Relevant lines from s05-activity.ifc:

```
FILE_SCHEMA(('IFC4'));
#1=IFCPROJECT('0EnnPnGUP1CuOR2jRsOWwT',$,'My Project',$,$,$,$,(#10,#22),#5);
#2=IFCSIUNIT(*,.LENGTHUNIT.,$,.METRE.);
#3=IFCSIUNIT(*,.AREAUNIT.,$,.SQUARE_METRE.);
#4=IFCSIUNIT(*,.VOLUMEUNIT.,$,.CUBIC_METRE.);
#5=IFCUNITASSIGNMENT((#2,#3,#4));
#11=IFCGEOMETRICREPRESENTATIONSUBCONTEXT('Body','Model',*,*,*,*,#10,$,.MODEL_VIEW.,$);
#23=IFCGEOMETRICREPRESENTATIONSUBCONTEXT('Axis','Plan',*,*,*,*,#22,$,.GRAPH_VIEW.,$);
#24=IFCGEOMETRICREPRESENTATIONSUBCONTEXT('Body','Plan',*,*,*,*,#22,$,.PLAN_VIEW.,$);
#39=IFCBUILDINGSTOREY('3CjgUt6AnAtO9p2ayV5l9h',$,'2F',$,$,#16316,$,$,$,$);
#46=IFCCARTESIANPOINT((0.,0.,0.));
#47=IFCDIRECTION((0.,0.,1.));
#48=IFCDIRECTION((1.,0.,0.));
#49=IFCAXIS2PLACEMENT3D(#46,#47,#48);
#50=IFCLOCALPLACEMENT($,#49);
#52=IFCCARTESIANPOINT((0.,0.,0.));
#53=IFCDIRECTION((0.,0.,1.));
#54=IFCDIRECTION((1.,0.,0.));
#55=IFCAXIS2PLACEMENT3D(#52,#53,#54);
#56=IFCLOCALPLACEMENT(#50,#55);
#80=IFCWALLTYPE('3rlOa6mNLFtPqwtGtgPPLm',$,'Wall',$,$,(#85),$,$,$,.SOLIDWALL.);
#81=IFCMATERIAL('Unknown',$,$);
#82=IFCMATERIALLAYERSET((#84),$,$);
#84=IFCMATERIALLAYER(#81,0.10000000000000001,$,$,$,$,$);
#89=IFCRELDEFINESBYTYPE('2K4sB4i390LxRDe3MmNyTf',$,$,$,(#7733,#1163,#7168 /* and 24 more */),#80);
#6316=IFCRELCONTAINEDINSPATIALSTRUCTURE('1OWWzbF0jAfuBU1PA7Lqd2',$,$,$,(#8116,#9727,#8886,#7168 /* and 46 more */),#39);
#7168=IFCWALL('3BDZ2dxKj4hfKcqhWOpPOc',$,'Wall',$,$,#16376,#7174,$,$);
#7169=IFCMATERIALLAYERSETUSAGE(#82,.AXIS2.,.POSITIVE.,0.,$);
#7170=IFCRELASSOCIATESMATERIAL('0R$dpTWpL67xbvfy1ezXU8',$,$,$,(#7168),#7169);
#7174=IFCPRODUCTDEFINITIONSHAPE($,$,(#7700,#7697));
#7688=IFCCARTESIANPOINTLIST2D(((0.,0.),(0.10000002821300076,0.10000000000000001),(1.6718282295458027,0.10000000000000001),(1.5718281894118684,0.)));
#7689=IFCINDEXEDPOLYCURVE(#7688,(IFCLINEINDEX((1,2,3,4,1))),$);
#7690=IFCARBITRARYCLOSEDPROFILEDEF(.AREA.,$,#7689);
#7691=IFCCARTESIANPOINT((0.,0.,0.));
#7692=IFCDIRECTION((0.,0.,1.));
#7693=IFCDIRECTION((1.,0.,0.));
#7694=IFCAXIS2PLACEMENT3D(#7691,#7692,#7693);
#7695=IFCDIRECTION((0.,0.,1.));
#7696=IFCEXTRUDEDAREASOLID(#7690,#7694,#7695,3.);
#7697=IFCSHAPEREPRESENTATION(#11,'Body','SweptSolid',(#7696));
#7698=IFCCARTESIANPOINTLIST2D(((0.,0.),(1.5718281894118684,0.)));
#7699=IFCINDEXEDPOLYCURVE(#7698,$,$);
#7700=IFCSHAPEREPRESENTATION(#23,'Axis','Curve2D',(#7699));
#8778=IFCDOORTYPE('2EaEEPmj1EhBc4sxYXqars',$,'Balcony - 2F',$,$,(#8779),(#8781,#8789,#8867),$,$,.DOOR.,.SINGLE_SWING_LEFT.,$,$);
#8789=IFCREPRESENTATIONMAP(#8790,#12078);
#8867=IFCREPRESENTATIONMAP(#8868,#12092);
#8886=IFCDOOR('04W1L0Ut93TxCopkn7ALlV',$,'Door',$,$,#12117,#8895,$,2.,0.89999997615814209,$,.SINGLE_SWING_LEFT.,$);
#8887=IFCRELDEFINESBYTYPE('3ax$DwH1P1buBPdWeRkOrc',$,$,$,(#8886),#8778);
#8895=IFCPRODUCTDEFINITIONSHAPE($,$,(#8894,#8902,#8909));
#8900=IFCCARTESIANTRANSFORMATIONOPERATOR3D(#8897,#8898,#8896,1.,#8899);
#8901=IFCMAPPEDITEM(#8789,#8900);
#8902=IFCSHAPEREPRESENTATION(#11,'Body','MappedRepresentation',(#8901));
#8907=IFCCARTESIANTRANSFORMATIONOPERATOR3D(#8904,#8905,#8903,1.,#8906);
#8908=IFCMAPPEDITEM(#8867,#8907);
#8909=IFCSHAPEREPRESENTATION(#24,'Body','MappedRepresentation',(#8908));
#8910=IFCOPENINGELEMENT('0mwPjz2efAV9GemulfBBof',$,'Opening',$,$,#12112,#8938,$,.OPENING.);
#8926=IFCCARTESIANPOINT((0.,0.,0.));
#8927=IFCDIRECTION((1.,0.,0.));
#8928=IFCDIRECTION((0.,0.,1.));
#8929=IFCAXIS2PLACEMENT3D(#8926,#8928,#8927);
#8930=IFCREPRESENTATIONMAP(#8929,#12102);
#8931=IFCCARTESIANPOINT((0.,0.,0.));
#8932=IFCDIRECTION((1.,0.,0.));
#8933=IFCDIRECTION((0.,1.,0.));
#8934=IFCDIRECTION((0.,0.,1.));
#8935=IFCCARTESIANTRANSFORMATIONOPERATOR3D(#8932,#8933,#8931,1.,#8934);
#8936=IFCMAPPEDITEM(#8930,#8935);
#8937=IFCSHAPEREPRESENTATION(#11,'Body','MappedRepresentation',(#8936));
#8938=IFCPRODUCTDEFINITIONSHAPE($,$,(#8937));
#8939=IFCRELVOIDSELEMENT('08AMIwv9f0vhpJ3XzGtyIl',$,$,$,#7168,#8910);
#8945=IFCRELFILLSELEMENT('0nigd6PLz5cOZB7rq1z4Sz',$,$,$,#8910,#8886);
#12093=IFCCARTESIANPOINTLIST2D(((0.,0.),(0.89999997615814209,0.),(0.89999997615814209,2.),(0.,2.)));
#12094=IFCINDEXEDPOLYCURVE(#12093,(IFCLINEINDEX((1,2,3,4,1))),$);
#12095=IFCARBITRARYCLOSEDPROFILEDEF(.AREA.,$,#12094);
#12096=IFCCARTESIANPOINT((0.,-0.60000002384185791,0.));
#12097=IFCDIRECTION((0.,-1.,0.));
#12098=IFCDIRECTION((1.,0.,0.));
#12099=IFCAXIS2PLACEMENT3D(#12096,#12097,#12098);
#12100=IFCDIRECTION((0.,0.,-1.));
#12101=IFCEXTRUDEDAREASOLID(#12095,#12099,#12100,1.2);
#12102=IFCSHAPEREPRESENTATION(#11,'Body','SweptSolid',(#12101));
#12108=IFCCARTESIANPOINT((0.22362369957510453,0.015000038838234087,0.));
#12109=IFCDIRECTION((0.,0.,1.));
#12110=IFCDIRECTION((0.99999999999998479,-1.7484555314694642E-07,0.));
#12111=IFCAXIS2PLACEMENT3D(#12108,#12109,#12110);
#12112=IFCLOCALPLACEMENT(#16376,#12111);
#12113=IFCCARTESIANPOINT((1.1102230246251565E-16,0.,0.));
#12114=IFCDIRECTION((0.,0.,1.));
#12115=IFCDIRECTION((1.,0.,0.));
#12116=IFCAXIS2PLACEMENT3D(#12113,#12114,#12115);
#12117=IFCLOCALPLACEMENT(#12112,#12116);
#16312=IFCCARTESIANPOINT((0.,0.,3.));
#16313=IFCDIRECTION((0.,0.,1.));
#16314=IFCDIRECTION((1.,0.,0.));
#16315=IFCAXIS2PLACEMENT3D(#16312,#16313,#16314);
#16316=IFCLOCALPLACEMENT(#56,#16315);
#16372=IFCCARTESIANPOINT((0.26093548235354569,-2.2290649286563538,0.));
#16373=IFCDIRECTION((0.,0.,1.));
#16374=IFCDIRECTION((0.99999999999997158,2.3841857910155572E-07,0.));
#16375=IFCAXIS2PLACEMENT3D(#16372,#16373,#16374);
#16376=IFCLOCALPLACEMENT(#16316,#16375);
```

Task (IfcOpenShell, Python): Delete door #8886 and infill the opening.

```python
import ifcopenshell
import ifcopenshell.api.feature
import ifcopenshell.api.root
import ifcopenshell.geom
import ifcopenshell.util.shape

model = ifcopenshell.open("s05-activity.ifc")
settings = ifcopenshell.geom.settings()


def volume(element):
    """Net volume in cubic metres, openings subtracted."""
    shape = ifcopenshell.geom.create_shape(settings, element)
    return ifcopenshell.util.shape.get_volume(shape.geometry)


door = model.by_id(8886)
opening = door.FillsVoids[0].RelatingOpeningElement
wall = opening.VoidsElements[0].RelatingBuildingElement
before = volume(wall)

ifcopenshell.api.root.remove_product(model, product=door)
ifcopenshell.api.feature.remove_feature(model, feature=opening)

after = volume(wall)

print(f"wall volume {before:.3f} -> {after:.3f} m3")

model.write("s05-activity-out.ifc")
```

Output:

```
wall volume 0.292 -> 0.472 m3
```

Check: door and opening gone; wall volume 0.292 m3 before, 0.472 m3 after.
